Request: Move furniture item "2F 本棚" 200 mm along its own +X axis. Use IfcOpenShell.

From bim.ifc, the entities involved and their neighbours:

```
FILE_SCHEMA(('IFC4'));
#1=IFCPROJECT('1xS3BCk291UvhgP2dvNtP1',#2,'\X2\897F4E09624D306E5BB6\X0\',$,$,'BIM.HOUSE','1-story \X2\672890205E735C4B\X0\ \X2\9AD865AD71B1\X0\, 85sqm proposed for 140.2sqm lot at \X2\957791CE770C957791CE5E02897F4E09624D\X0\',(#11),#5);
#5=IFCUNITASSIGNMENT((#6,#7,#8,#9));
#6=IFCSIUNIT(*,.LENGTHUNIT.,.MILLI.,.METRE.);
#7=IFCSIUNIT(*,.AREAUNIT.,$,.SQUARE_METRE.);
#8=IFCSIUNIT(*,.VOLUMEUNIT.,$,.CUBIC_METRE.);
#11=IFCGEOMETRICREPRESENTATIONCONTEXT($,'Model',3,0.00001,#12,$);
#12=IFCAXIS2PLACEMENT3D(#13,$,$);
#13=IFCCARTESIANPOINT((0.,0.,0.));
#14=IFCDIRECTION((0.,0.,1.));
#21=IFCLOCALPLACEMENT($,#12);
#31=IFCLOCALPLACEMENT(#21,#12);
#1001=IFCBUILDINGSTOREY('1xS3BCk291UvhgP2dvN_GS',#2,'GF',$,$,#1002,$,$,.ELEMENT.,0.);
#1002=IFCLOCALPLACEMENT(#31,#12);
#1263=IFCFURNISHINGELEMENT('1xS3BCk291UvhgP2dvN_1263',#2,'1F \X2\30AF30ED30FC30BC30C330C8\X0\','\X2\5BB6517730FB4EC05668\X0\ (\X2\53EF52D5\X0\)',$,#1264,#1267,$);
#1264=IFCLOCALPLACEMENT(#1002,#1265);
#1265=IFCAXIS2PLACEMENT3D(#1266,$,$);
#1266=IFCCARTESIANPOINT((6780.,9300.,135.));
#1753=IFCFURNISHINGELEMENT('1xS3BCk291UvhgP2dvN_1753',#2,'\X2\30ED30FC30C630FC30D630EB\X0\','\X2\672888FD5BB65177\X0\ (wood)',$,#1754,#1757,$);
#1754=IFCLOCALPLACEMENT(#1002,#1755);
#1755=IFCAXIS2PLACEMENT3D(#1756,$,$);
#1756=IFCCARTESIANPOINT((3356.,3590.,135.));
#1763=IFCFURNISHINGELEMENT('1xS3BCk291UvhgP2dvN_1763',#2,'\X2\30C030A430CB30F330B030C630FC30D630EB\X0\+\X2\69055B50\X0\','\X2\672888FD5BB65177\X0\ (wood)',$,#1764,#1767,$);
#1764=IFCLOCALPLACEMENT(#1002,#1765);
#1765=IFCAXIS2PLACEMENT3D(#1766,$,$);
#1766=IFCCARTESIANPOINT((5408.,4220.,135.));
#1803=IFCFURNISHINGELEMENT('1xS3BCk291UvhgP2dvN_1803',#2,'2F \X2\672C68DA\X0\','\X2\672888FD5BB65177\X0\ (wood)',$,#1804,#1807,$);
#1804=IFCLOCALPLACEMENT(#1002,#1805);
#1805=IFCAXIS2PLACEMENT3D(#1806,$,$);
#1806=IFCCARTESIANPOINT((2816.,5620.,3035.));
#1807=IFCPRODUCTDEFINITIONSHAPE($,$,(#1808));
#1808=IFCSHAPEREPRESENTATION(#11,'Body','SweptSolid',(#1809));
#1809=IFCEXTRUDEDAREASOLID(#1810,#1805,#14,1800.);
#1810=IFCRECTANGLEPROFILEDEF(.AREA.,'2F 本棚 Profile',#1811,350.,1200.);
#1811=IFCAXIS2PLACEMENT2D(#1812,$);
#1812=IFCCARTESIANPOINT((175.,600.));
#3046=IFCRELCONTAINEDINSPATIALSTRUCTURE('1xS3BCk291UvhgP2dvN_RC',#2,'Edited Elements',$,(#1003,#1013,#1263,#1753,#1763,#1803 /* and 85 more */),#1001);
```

```python
import ifcopenshell
import ifcopenshell.api.geometry
import ifcopenshell.util.placement

model = ifcopenshell.open("bim.ifc")

item = model.by_guid("1xS3BCk291UvhgP2dvN_1803")
matrix = ifcopenshell.util.placement.get_local_placement(item.ObjectPlacement)
matrix[:3, 3] += matrix[:3, 0] * 200.0
ifcopenshell.api.geometry.edit_object_placement(model, product=item, matrix=matrix, is_si=False)

print(ifcopenshell.util.placement.get_local_placement(item.ObjectPlacement).round(3) + 0.0)

model.write("bim-out.ifc")
```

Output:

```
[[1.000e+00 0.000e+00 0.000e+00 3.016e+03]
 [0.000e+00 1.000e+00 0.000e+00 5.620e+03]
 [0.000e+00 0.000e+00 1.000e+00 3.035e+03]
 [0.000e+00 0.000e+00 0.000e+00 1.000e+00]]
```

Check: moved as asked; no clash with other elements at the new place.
